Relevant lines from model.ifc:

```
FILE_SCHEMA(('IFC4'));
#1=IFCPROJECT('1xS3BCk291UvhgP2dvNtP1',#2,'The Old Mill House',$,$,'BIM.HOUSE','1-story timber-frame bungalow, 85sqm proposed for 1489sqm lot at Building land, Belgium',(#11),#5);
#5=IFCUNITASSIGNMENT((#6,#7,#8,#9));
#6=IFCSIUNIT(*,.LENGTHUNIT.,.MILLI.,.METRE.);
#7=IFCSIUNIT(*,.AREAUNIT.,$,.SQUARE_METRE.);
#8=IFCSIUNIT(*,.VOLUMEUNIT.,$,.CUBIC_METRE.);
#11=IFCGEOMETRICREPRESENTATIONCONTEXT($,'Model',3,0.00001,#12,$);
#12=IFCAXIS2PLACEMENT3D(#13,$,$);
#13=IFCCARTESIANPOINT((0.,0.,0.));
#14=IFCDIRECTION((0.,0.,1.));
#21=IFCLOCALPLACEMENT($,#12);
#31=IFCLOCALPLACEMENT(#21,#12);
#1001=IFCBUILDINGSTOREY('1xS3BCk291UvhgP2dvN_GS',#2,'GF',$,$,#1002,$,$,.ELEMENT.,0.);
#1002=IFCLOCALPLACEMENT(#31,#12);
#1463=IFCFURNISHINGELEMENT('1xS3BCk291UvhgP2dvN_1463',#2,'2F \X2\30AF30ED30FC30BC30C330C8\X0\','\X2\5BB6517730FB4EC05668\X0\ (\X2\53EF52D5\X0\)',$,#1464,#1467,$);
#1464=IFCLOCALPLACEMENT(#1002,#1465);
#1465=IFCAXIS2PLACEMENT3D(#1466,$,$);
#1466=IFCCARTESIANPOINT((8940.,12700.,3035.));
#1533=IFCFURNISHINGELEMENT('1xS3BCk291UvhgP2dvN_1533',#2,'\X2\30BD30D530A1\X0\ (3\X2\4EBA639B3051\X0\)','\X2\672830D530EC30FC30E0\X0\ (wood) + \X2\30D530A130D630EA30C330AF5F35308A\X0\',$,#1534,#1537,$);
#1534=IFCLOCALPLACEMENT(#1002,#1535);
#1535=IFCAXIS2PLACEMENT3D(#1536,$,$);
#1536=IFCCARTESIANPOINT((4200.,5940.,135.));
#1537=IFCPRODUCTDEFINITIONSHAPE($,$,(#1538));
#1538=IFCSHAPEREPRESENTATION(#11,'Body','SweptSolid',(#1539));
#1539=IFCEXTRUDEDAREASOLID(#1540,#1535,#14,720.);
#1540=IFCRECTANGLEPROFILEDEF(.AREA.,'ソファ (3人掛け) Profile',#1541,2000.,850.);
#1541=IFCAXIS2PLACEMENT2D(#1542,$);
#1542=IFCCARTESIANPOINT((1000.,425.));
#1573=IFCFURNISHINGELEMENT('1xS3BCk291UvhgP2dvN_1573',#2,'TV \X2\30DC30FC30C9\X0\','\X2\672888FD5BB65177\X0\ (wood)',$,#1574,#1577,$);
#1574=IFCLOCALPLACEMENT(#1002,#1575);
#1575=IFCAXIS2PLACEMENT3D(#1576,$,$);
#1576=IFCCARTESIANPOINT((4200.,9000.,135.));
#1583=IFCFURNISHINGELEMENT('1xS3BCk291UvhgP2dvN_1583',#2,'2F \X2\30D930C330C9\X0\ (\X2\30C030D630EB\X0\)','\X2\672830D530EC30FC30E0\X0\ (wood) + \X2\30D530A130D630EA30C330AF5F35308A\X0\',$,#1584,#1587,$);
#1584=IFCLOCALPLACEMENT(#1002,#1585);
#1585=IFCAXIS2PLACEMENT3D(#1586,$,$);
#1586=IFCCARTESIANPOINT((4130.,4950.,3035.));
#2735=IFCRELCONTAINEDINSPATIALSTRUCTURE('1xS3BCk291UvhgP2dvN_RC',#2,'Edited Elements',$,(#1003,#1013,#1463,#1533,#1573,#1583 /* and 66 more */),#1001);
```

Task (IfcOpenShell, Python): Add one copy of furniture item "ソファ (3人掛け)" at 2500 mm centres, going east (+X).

```python
import numpy as np
import ifcopenshell
import ifcopenshell.api.geometry
import ifcopenshell.api.root
import ifcopenshell.util.element
import ifcopenshell.util.placement
import ifcopenshell.util.unit

model = ifcopenshell.open("model.ifc")
unit_scale = ifcopenshell.util.unit.calculate_unit_scale(model)


def reuse_history(source, copy):
    """copy_class also copies each property set's owner history, people and application; keep the originals."""
    for rel in copy.IsDefinedBy:
        if rel.is_a("IfcRelDefinesByProperties") and (history := rel.RelatingPropertyDefinition.OwnerHistory):
            rel.RelatingPropertyDefinition.OwnerHistory = source.OwnerHistory
            ifcopenshell.util.element.remove_deep2(model, history)


source = model.by_guid("1xS3BCk291UvhgP2dvN_1533")
base = ifcopenshell.util.placement.get_local_placement(source.ObjectPlacement)
step = np.array([1.0, 0.0, 0.0]) * 2.5 / unit_scale

for i in range(1, 2):
    copy = ifcopenshell.api.root.copy_class(model, product=source)
    copy.Representation = ifcopenshell.util.element.copy_deep(
        model, source.Representation, exclude=["IfcGeometricRepresentationContext", "IfcRepresentationMap"]
    )
    reuse_history(source, copy)
    matrix = base.copy()
    matrix[:3, 3] += i * step
    print("added at", matrix[:3, 3].round(3) + 0.0)
    ifcopenshell.api.geometry.edit_object_placement(model, product=copy, matrix=matrix, is_si=False)

model.write("model_edited.ifc")
```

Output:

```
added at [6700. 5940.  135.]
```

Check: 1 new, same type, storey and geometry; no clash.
